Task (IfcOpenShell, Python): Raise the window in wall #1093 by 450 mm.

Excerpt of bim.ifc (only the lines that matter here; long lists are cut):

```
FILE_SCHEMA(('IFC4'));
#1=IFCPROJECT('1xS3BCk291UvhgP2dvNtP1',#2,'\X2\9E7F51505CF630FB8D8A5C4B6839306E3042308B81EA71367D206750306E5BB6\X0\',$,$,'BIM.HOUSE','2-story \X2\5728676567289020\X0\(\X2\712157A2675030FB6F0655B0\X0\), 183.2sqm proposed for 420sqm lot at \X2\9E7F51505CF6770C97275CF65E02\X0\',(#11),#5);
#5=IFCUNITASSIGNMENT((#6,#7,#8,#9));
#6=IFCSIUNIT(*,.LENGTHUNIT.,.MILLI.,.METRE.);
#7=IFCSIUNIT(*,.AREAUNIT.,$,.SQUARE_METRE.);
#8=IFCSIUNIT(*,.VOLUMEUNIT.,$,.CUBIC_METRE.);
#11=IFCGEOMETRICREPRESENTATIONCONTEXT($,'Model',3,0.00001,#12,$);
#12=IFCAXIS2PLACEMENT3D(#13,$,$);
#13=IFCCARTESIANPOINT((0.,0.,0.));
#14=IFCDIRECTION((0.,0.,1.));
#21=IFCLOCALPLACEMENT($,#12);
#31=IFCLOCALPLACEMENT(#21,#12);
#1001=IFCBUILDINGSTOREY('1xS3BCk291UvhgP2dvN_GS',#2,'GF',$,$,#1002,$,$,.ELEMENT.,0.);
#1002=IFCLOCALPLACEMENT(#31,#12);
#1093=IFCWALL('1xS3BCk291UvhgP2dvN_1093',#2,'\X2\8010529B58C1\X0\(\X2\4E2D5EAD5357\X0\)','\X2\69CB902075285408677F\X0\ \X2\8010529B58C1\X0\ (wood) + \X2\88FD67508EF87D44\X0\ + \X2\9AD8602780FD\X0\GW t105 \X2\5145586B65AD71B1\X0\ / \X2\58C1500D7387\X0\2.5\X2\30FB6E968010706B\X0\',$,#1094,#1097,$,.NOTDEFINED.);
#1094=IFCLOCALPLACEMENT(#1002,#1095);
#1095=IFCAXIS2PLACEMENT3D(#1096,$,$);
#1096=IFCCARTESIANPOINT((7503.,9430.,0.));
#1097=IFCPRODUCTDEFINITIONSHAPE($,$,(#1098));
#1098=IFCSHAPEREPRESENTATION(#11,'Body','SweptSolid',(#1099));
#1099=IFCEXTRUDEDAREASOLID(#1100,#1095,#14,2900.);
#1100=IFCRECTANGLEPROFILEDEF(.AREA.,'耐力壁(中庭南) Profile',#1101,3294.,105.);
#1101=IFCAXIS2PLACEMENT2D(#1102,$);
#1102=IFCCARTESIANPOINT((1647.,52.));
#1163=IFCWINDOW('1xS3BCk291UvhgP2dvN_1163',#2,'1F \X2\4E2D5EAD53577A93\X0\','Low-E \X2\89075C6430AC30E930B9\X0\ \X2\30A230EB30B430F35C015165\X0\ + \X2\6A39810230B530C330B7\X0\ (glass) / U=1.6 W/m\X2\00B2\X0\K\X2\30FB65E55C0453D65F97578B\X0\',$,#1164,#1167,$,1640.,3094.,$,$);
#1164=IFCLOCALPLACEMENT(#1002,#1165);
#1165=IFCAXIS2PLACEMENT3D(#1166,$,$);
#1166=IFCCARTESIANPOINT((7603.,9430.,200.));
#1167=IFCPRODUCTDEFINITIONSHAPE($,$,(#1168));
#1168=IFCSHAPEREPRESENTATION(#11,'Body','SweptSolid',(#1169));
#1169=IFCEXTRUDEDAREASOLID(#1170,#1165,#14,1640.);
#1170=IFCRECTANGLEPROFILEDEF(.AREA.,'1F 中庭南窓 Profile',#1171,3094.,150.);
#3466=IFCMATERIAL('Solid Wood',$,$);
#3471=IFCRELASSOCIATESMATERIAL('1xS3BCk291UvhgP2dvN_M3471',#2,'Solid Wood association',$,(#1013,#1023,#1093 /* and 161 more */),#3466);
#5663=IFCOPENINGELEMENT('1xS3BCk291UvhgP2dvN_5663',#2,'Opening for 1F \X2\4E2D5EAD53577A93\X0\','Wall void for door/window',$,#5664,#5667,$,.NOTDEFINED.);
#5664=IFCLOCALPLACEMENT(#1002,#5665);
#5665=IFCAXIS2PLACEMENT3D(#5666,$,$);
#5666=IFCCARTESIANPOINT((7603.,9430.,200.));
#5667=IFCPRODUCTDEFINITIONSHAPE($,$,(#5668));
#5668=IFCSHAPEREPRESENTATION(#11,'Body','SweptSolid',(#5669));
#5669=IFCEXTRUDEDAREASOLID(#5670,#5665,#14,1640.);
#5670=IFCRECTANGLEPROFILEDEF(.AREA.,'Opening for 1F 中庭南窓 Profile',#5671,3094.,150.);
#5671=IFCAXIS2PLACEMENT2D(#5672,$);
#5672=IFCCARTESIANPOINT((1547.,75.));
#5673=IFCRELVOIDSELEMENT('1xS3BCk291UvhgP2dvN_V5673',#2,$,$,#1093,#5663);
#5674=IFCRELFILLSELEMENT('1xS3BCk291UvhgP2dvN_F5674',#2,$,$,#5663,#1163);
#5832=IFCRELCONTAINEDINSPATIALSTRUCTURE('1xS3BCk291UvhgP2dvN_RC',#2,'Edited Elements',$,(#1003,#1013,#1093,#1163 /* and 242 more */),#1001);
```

```python
import numpy as np
import ifcopenshell
import ifcopenshell.api.geometry
import ifcopenshell.util.placement
import ifcopenshell.util.unit

model = ifcopenshell.open("bim.ifc")
unit_scale = ifcopenshell.util.unit.calculate_unit_scale(model)

window = model.by_guid("1xS3BCk291UvhgP2dvN_1163")
opening = window.FillsVoids[0].RelatingOpeningElement
dz = 0.45 / unit_scale

shift = np.array([0.0, 0.0, dz])
# The window is not placed relative to its opening, so move both.
for product in (opening, window):
    matrix = ifcopenshell.util.placement.get_local_placement(product.ObjectPlacement)
    matrix[:3, 3] += shift
    ifcopenshell.api.geometry.edit_object_placement(model, product=product, matrix=matrix, is_si=False)

print(f"moved by {dz * unit_scale:+.3f} m")

model.write("bim_edited.ifc")
```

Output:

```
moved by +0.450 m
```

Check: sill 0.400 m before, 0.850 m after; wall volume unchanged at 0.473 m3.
